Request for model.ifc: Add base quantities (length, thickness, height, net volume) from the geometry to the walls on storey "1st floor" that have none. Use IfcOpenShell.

First a look at what the model holds.

```python
import ifcopenshell
import ifcopenshell.util.element
import ifcopenshell.util.unit

model = ifcopenshell.open("model.ifc")
print(model.schema)
for unit_type in ("LENGTHUNIT", "AREAUNIT", "VOLUMEUNIT"):
    print(unit_type, ifcopenshell.util.unit.calculate_unit_scale(model, unit_type))
storey = next(s for s in model.by_type("IfcBuildingStorey") if s.Name == "1st floor")
walls = [e for e in ifcopenshell.util.element.get_decomposition(storey) if e.is_a("IfcWall")]
for e in sorted(walls, key=lambda e: e.id()):
    print(e.id(), e.is_a(), e.Name, list(ifcopenshell.util.element.get_psets(e, qtos_only=True)), sep=" | ")
```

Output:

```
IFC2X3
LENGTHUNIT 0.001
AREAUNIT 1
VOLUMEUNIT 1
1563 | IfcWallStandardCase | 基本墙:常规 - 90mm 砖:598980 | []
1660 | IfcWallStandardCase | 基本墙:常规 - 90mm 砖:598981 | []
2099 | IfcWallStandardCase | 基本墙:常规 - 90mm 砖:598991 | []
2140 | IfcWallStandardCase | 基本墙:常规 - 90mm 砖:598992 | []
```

```python
import ifcopenshell
import ifcopenshell.api.pset
import ifcopenshell.geom
import ifcopenshell.util.element
import ifcopenshell.util.shape
import ifcopenshell.util.unit

model = ifcopenshell.open("model.ifc")
unit_scale = ifcopenshell.util.unit.calculate_unit_scale(model)
volume_scale = ifcopenshell.util.unit.calculate_unit_scale(model, "VOLUMEUNIT")
settings = ifcopenshell.geom.settings()

storey = next(s for s in model.by_type("IfcBuildingStorey") if s.Name == "1st floor")
walls = [e for e in ifcopenshell.util.element.get_decomposition(storey) if e.is_a("IfcWall")]

for e in sorted(walls, key=lambda e: e.id()):
    if ifcopenshell.util.element.get_psets(e, qtos_only=True, should_inherit=False):
        continue
    # Geometry comes back in metres, in the element's own axes.
    shape = ifcopenshell.geom.create_shape(settings, e)
    values = {
        "Length": ifcopenshell.util.shape.get_x(shape.geometry) / unit_scale,
        "Width": ifcopenshell.util.shape.get_y(shape.geometry) / unit_scale,
        "Height": ifcopenshell.util.shape.get_z(shape.geometry) / unit_scale,
        "NetVolume": ifcopenshell.util.shape.get_volume(shape.geometry) / volume_scale,
    }
    qto = ifcopenshell.api.pset.add_qto(model, product=e, name="BaseQuantities")
    ifcopenshell.api.pset.edit_qto(model, qto=qto, properties=values)
    print(e.id(), {k: round(v, 3) for k, v in values.items()})

model.write("model-out.ifc")
```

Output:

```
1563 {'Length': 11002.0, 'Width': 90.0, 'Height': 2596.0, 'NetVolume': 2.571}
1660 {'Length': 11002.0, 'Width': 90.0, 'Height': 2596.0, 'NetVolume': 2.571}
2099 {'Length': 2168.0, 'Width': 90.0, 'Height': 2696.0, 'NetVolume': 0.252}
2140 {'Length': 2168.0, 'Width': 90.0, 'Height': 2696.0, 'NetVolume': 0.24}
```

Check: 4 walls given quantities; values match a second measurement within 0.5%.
